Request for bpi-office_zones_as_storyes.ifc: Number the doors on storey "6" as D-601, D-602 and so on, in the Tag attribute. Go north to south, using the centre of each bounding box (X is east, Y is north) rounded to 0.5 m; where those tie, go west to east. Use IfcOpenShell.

First a look at what the model holds.

```python
import ifcopenshell
import ifcopenshell.util.element
import ifcopenshell.util.placement

model = ifcopenshell.open("bpi-office_zones_as_storyes.ifc")
print(model.schema)
storey = next(s for s in model.by_type("IfcBuildingStorey") if s.Name == "6")
doors = [e for e in ifcopenshell.util.element.get_decomposition(storey) if e.is_a("IfcDoor")]
for e in sorted(doors, key=lambda e: e.id()):
    origin = ifcopenshell.util.placement.get_local_placement(e.ObjectPlacement)[:3, 3]
    print(e.id(), e.Tag, e.Name, origin.round(2) + 0.0, sep=" | ")
```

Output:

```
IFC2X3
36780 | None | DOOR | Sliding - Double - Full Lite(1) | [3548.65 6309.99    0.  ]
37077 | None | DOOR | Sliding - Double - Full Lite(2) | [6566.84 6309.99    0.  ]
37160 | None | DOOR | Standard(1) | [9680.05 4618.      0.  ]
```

```python
import ifcopenshell
import ifcopenshell.geom
import ifcopenshell.util.element
import ifcopenshell.util.shape

model = ifcopenshell.open("bpi-office_zones_as_storyes.ifc")
settings = ifcopenshell.geom.settings()
settings.set("use-world-coords", True)


def centre(element):
    shape = ifcopenshell.geom.create_shape(settings, element)
    return ifcopenshell.util.shape.get_bbox_centroid(shape.geometry)


storey = next(s for s in model.by_type("IfcBuildingStorey") if s.Name == "6")
doors = [e for e in ifcopenshell.util.element.get_decomposition(storey) if e.is_a("IfcDoor")]

# Insertion points can sit at a corner or the storey origin, so sort by the geometry (in metres).
centres = {e: centre(e) for e in doors}
doors.sort(key=lambda e: (-round(centres[e][1] / 0.5), centres[e][0]))

for i, e in enumerate(doors, start=1):
    number = f"D-6{i:02d}"
    e.Tag = number
    print(e.id(), number)

model.write("bpi-office_zones_as_storyes_edited.ifc")
```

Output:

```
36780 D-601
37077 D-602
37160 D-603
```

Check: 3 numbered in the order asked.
